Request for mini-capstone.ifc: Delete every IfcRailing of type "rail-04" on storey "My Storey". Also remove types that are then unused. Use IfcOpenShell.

First a look at what the model holds.

```python
import ifcopenshell
import ifcopenshell.util.element

model = ifcopenshell.open("mini-capstone.ifc")
print(model.schema)
storey = next(s for s in model.by_type("IfcBuildingStorey") if s.Name == "My Storey")
railings = [e for e in ifcopenshell.util.element.get_decomposition(storey) if e.is_a("IfcRailing")]
seen = {}
for e in railings:
    element_type = ifcopenshell.util.element.get_type(e)
    name = element_type.Name if element_type not in (None, e) else None
    seen[name] = seen.get(name, 0) + 1
for name, count in sorted(seen.items(), key=str):
    print(count, "x", name)
```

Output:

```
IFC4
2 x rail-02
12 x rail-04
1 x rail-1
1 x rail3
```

```python
import ifcopenshell
import ifcopenshell.api.root
import ifcopenshell.util.element

model = ifcopenshell.open("mini-capstone.ifc")

storey = next(s for s in model.by_type("IfcBuildingStorey") if s.Name == "My Storey")
railings = [e for e in ifcopenshell.util.element.get_decomposition(storey) if e.is_a("IfcRailing")]
targets = [e for e in railings if (t := ifcopenshell.util.element.get_type(e)) not in (None, e) and t.Name == "rail-04"]
types = {ifcopenshell.util.element.get_type(e) for e in targets} - {None, *targets}

for e in targets:
    ifcopenshell.api.root.remove_product(model, product=e)
print(len(targets), "removed")

unused = [t for t in types if not ifcopenshell.util.element.get_types(t)]
for t in unused:
    ifcopenshell.api.root.remove_product(model, product=t)
print(len(unused), "unused types removed")

model.write("mini-capstone_rev.ifc")
```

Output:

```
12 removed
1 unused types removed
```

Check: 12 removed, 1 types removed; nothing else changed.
